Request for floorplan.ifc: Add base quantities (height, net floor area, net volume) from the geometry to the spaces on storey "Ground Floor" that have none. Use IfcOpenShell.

First a look at what the model holds.

```python
import ifcopenshell
import ifcopenshell.util.element
import ifcopenshell.util.unit

model = ifcopenshell.open("floorplan.ifc")
print(model.schema)
for unit_type in ("LENGTHUNIT", "AREAUNIT", "VOLUMEUNIT"):
    print(unit_type, ifcopenshell.util.unit.calculate_unit_scale(model, unit_type))
storey = next(s for s in model.by_type("IfcBuildingStorey") if s.Name == "Ground Floor")
spaces = [e for e in ifcopenshell.util.element.get_decomposition(storey) if e.is_a("IfcSpace")]
for e in sorted(spaces, key=lambda e: e.id()):
    print(e.id(), e.is_a(), e.Name, list(ifcopenshell.util.element.get_psets(e, qtos_only=True)), sep=" | ")
```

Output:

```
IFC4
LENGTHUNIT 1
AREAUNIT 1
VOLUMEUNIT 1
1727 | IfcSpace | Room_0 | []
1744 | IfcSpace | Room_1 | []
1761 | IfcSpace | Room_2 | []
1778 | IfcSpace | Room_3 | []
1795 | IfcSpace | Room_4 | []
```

```python
import ifcopenshell
import ifcopenshell.api.pset
import ifcopenshell.geom
import ifcopenshell.util.element
import ifcopenshell.util.shape
import ifcopenshell.util.unit

model = ifcopenshell.open("floorplan.ifc")
unit_scale = ifcopenshell.util.unit.calculate_unit_scale(model)
area_scale = ifcopenshell.util.unit.calculate_unit_scale(model, "AREAUNIT")
volume_scale = ifcopenshell.util.unit.calculate_unit_scale(model, "VOLUMEUNIT")
settings = ifcopenshell.geom.settings()

storey = next(s for s in model.by_type("IfcBuildingStorey") if s.Name == "Ground Floor")
spaces = [e for e in ifcopenshell.util.element.get_decomposition(storey) if e.is_a("IfcSpace")]

for e in sorted(spaces, key=lambda e: e.id()):
    if ifcopenshell.util.element.get_psets(e, qtos_only=True, should_inherit=False):
        continue
    # Geometry comes back in metres, in the element's own axes.
    shape = ifcopenshell.geom.create_shape(settings, e)
    values = {
        "Height": ifcopenshell.util.shape.get_z(shape.geometry) / unit_scale,
        "NetFloorArea": ifcopenshell.util.shape.get_footprint_area(shape.geometry) / area_scale,
        "NetVolume": ifcopenshell.util.shape.get_volume(shape.geometry) / volume_scale,
    }
    qto = ifcopenshell.api.pset.add_qto(model, product=e, name="Qto_SpaceBaseQuantities")
    ifcopenshell.api.pset.edit_qto(model, qto=qto, properties=values)
    print(e.id(), {k: round(v, 3) for k, v in values.items()})

model.write("floorplan_rev.ifc")
```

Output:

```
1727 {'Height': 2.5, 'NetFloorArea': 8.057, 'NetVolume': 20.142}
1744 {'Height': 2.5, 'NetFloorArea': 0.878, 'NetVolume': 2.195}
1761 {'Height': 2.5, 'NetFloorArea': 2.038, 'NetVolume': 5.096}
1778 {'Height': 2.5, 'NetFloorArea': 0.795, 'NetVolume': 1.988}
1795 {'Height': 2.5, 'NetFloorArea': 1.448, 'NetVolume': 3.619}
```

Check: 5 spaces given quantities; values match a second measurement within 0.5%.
